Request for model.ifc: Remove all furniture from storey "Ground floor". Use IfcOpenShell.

First a look at what the model holds.

```python
import ifcopenshell
import ifcopenshell.util.element

model = ifcopenshell.open("model.ifc")
print(model.schema)
storey = next(s for s in model.by_type("IfcBuildingStorey") if s.Name == "Ground floor")
furniture = [e for e in ifcopenshell.util.element.get_decomposition(storey) if e.is_a("IfcFurnishingElement")]
seen = {}
for e in furniture:
    element_type = ifcopenshell.util.element.get_type(e)
    name = element_type.Name if element_type not in (None, e) else None
    seen[name] = seen.get(name, 0) + 1
for name, count in sorted(seen.items(), key=str):
    print(count, "x", name)
```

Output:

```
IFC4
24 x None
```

```python
import ifcopenshell
import ifcopenshell.api.root
import ifcopenshell.util.element

model = ifcopenshell.open("model.ifc")

storey = next(s for s in model.by_type("IfcBuildingStorey") if s.Name == "Ground floor")
furniture = [e for e in ifcopenshell.util.element.get_decomposition(storey) if e.is_a("IfcFurnishingElement")]

for e in furniture:
    ifcopenshell.api.root.remove_product(model, product=e)
print(len(furniture), "removed")

model.write("model_v2.ifc")
```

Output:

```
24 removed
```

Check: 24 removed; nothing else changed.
